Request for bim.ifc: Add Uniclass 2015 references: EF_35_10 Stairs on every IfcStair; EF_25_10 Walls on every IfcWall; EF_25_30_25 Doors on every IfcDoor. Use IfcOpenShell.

First a look at what the model holds.

```python
import ifcopenshell

model = ifcopenshell.open("bim.ifc")
print(model.schema)
print("classifications:", [c.Name for c in model.by_type("IfcClassification")])
for ifc_class in ("IfcDoor", "IfcRoof", "IfcStair", "IfcWall", "IfcWindow"):
    print(ifc_class, len(model.by_type(ifc_class)))
```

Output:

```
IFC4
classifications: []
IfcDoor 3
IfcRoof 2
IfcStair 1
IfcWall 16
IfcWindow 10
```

```python
import ifcopenshell
import ifcopenshell.api.classification

model = ifcopenshell.open("bim.ifc")

system = ifcopenshell.api.classification.add_classification(model, classification="Uniclass 2015")

codes = {
    "IfcStair": ("EF_35_10", "Stairs"),
    "IfcWall": ("EF_25_10", "Walls"),
    "IfcDoor": ("EF_25_30_25", "Doors"),
}
for ifc_class, (code, name) in codes.items():
    products = model.by_type(ifc_class)
    ifcopenshell.api.classification.add_reference(
        model, products=products, classification=system, identification=code, name=name
    )
    print(code, len(products))

model.write("bim_edited.ifc")
```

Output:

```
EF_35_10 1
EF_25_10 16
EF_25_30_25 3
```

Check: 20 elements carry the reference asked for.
